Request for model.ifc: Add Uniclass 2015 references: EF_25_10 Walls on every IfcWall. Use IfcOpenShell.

First a look at what the model holds.

```python
import ifcopenshell

model = ifcopenshell.open("model.ifc")
print(model.schema)
print("classifications:", [c.Name for c in model.by_type("IfcClassification")])
for ifc_class in ("IfcDoor", "IfcRoof", "IfcStair", "IfcWall", "IfcWindow"):
    print(ifc_class, len(model.by_type(ifc_class)))
```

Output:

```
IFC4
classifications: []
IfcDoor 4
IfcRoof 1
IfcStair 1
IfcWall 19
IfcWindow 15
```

```python
import ifcopenshell
import ifcopenshell.api.classification

model = ifcopenshell.open("model.ifc")

system = ifcopenshell.api.classification.add_classification(model, classification="Uniclass 2015")

codes = {
    "IfcWall": ("EF_25_10", "Walls"),
}
for ifc_class, (code, name) in codes.items():
    products = model.by_type(ifc_class)
    ifcopenshell.api.classification.add_reference(
        model, products=products, classification=system, identification=code, name=name
    )
    print(code, len(products))

model.write("model_v2.ifc")
```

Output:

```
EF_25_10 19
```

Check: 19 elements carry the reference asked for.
